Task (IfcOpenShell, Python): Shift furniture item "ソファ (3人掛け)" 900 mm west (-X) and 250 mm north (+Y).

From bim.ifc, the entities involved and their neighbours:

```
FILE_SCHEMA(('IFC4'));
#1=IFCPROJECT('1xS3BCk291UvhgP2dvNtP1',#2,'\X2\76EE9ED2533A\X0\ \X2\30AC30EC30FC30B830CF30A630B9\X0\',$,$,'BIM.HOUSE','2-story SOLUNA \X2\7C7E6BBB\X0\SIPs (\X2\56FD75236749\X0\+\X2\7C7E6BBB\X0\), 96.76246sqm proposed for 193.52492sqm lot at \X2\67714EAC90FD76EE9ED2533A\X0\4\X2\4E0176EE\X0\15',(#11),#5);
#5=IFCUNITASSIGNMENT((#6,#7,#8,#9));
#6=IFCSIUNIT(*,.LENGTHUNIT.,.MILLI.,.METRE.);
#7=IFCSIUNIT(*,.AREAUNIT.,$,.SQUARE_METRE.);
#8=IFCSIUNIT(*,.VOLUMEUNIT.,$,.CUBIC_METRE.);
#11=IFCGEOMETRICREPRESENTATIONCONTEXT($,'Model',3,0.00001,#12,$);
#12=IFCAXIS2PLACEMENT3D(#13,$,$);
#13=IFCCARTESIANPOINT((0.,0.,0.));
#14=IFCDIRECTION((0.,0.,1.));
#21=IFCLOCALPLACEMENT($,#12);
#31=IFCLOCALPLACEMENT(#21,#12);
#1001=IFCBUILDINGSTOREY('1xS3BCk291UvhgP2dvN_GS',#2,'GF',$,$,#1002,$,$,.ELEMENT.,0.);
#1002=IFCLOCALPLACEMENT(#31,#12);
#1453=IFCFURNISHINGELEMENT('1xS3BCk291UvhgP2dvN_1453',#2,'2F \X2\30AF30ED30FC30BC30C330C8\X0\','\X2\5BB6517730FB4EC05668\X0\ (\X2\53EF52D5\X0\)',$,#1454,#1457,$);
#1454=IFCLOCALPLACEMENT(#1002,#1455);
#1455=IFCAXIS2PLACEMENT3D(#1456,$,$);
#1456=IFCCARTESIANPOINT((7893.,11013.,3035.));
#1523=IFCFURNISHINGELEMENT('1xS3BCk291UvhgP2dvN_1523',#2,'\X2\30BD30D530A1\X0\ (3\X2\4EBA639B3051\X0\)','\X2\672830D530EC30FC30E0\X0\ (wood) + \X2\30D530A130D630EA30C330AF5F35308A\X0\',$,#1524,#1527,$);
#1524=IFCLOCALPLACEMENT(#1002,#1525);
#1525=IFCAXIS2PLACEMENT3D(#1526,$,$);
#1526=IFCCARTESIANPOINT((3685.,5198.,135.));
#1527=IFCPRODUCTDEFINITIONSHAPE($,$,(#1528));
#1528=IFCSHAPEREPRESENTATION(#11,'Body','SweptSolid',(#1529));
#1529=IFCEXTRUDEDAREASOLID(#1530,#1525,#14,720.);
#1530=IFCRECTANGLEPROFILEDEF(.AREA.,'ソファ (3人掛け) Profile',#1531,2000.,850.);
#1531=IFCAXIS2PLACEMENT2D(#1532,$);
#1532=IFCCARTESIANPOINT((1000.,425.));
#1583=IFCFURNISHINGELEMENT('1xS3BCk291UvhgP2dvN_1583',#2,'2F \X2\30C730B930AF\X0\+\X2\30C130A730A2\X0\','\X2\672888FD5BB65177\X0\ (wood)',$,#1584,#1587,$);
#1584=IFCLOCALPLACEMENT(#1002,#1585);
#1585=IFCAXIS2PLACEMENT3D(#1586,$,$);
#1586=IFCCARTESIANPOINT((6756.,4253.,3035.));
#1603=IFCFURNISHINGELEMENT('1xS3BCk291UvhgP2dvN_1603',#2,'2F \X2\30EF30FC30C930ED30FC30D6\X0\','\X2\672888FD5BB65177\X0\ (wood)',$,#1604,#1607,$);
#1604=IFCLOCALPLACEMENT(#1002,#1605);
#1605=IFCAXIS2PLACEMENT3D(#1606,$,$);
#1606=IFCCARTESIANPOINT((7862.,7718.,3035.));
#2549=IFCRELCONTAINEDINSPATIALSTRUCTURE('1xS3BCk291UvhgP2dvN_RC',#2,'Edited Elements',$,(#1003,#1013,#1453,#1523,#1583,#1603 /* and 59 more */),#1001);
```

```python
import ifcopenshell
import ifcopenshell.api.geometry
import ifcopenshell.util.placement

model = ifcopenshell.open("bim.ifc")

item = model.by_guid("1xS3BCk291UvhgP2dvN_1523")
matrix = ifcopenshell.util.placement.get_local_placement(item.ObjectPlacement)
matrix[0, 3] -= 900.0
matrix[1, 3] += 250.0
ifcopenshell.api.geometry.edit_object_placement(model, product=item, matrix=matrix, is_si=False)

print(ifcopenshell.util.placement.get_local_placement(item.ObjectPlacement).round(3) + 0.0)

model.write("bim_v2.ifc")
```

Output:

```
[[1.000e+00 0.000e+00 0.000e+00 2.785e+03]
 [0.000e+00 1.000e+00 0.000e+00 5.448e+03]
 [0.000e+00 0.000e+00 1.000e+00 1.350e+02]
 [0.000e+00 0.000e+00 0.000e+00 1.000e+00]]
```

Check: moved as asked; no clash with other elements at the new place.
